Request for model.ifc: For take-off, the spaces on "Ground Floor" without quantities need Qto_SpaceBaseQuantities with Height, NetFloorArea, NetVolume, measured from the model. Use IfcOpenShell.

First a look at what the model holds.

```python
import ifcopenshell
import ifcopenshell.util.element
import ifcopenshell.util.unit

model = ifcopenshell.open("model.ifc")
print(model.schema)
for unit_type in ("LENGTHUNIT", "AREAUNIT", "VOLUMEUNIT"):
    print(unit_type, ifcopenshell.util.unit.calculate_unit_scale(model, unit_type))
storey = next(s for s in model.by_type("IfcBuildingStorey") if s.Name == "Ground Floor")
spaces = [e for e in ifcopenshell.util.element.get_decomposition(storey) if e.is_a("IfcSpace")]
for e in sorted(spaces, key=lambda e: e.id()):
    print(e.id(), e.is_a(), e.Name, list(ifcopenshell.util.element.get_psets(e, qtos_only=True)), sep=" | ")
```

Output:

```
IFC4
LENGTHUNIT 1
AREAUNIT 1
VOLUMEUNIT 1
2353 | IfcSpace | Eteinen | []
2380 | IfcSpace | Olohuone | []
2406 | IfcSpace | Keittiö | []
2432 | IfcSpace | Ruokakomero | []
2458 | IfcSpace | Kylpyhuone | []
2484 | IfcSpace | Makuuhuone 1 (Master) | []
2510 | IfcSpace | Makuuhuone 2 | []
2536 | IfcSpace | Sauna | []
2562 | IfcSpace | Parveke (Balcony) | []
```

```python
import ifcopenshell
import ifcopenshell.api.pset
import ifcopenshell.geom
import ifcopenshell.util.element
import ifcopenshell.util.shape
import ifcopenshell.util.unit

model = ifcopenshell.open("model.ifc")
unit_scale = ifcopenshell.util.unit.calculate_unit_scale(model)
area_scale = ifcopenshell.util.unit.calculate_unit_scale(model, "AREAUNIT")
volume_scale = ifcopenshell.util.unit.calculate_unit_scale(model, "VOLUMEUNIT")
settings = ifcopenshell.geom.settings()

storey = next(s for s in model.by_type("IfcBuildingStorey") if s.Name == "Ground Floor")
spaces = [e for e in ifcopenshell.util.element.get_decomposition(storey) if e.is_a("IfcSpace")]

for e in sorted(spaces, key=lambda e: e.id()):
    if ifcopenshell.util.element.get_psets(e, qtos_only=True, should_inherit=False):
        continue
    # Geometry comes back in metres, in the element's own axes.
    shape = ifcopenshell.geom.create_shape(settings, e)
    values = {
        "Height": ifcopenshell.util.shape.get_z(shape.geometry) / unit_scale,
        "NetFloorArea": ifcopenshell.util.shape.get_footprint_area(shape.geometry) / area_scale,
        "NetVolume": ifcopenshell.util.shape.get_volume(shape.geometry) / volume_scale,
    }
    qto = ifcopenshell.api.pset.add_qto(model, product=e, name="Qto_SpaceBaseQuantities")
    ifcopenshell.api.pset.edit_qto(model, qto=qto, properties=values)
    print(e.id(), {k: round(v, 3) for k, v in values.items()})

model.write("model_rev.ifc")
```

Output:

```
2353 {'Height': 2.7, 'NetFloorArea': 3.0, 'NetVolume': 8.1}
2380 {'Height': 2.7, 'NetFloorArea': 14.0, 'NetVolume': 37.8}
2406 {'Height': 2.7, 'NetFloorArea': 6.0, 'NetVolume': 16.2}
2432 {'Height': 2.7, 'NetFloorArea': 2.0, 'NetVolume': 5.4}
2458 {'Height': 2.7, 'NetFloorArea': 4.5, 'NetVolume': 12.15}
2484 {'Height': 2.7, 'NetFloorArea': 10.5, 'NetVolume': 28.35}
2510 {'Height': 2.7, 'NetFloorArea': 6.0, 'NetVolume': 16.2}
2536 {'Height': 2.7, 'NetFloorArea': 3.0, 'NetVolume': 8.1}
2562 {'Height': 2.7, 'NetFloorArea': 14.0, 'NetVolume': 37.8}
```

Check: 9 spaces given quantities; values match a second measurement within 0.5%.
